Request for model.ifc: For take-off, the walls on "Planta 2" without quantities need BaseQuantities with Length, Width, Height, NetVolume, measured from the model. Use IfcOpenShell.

First a look at what the model holds.

```python
import ifcopenshell
import ifcopenshell.util.element
import ifcopenshell.util.unit

model = ifcopenshell.open("model.ifc")
print(model.schema)
for unit_type in ("LENGTHUNIT", "AREAUNIT", "VOLUMEUNIT"):
    print(unit_type, ifcopenshell.util.unit.calculate_unit_scale(model, unit_type))
storey = next(s for s in model.by_type("IfcBuildingStorey") if s.Name == "Planta 2")
walls = [e for e in ifcopenshell.util.element.get_decomposition(storey) if e.is_a("IfcWall")]
for e in sorted(walls, key=lambda e: e.id()):
    print(e.id(), e.is_a(), e.Name, list(ifcopenshell.util.element.get_psets(e, qtos_only=True)), sep=" | ")
```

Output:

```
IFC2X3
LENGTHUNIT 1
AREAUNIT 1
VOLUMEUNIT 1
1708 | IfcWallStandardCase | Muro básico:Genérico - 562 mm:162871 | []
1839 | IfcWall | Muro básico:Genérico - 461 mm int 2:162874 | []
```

```python
import ifcopenshell
import ifcopenshell.api.pset
import ifcopenshell.geom
import ifcopenshell.util.element
import ifcopenshell.util.shape
import ifcopenshell.util.unit

model = ifcopenshell.open("model.ifc")
unit_scale = ifcopenshell.util.unit.calculate_unit_scale(model)
volume_scale = ifcopenshell.util.unit.calculate_unit_scale(model, "VOLUMEUNIT")
settings = ifcopenshell.geom.settings()

storey = next(s for s in model.by_type("IfcBuildingStorey") if s.Name == "Planta 2")
walls = [e for e in ifcopenshell.util.element.get_decomposition(storey) if e.is_a("IfcWall")]

for e in sorted(walls, key=lambda e: e.id()):
    if ifcopenshell.util.element.get_psets(e, qtos_only=True, should_inherit=False):
        continue
    # Geometry comes back in metres, in the element's own axes.
    shape = ifcopenshell.geom.create_shape(settings, e)
    values = {
        "Length": ifcopenshell.util.shape.get_x(shape.geometry) / unit_scale,
        "Width": ifcopenshell.util.shape.get_y(shape.geometry) / unit_scale,
        "Height": ifcopenshell.util.shape.get_z(shape.geometry) / unit_scale,
        "NetVolume": ifcopenshell.util.shape.get_volume(shape.geometry) / volume_scale,
    }
    qto = ifcopenshell.api.pset.add_qto(model, product=e, name="BaseQuantities")
    ifcopenshell.api.pset.edit_qto(model, qto=qto, properties=values)
    print(e.id(), {k: round(v, 3) for k, v in values.items()})

model.write("model_v2.ifc")
```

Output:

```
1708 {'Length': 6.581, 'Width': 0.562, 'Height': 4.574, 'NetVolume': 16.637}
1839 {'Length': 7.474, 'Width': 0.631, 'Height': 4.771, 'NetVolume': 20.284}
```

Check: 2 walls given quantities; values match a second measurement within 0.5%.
